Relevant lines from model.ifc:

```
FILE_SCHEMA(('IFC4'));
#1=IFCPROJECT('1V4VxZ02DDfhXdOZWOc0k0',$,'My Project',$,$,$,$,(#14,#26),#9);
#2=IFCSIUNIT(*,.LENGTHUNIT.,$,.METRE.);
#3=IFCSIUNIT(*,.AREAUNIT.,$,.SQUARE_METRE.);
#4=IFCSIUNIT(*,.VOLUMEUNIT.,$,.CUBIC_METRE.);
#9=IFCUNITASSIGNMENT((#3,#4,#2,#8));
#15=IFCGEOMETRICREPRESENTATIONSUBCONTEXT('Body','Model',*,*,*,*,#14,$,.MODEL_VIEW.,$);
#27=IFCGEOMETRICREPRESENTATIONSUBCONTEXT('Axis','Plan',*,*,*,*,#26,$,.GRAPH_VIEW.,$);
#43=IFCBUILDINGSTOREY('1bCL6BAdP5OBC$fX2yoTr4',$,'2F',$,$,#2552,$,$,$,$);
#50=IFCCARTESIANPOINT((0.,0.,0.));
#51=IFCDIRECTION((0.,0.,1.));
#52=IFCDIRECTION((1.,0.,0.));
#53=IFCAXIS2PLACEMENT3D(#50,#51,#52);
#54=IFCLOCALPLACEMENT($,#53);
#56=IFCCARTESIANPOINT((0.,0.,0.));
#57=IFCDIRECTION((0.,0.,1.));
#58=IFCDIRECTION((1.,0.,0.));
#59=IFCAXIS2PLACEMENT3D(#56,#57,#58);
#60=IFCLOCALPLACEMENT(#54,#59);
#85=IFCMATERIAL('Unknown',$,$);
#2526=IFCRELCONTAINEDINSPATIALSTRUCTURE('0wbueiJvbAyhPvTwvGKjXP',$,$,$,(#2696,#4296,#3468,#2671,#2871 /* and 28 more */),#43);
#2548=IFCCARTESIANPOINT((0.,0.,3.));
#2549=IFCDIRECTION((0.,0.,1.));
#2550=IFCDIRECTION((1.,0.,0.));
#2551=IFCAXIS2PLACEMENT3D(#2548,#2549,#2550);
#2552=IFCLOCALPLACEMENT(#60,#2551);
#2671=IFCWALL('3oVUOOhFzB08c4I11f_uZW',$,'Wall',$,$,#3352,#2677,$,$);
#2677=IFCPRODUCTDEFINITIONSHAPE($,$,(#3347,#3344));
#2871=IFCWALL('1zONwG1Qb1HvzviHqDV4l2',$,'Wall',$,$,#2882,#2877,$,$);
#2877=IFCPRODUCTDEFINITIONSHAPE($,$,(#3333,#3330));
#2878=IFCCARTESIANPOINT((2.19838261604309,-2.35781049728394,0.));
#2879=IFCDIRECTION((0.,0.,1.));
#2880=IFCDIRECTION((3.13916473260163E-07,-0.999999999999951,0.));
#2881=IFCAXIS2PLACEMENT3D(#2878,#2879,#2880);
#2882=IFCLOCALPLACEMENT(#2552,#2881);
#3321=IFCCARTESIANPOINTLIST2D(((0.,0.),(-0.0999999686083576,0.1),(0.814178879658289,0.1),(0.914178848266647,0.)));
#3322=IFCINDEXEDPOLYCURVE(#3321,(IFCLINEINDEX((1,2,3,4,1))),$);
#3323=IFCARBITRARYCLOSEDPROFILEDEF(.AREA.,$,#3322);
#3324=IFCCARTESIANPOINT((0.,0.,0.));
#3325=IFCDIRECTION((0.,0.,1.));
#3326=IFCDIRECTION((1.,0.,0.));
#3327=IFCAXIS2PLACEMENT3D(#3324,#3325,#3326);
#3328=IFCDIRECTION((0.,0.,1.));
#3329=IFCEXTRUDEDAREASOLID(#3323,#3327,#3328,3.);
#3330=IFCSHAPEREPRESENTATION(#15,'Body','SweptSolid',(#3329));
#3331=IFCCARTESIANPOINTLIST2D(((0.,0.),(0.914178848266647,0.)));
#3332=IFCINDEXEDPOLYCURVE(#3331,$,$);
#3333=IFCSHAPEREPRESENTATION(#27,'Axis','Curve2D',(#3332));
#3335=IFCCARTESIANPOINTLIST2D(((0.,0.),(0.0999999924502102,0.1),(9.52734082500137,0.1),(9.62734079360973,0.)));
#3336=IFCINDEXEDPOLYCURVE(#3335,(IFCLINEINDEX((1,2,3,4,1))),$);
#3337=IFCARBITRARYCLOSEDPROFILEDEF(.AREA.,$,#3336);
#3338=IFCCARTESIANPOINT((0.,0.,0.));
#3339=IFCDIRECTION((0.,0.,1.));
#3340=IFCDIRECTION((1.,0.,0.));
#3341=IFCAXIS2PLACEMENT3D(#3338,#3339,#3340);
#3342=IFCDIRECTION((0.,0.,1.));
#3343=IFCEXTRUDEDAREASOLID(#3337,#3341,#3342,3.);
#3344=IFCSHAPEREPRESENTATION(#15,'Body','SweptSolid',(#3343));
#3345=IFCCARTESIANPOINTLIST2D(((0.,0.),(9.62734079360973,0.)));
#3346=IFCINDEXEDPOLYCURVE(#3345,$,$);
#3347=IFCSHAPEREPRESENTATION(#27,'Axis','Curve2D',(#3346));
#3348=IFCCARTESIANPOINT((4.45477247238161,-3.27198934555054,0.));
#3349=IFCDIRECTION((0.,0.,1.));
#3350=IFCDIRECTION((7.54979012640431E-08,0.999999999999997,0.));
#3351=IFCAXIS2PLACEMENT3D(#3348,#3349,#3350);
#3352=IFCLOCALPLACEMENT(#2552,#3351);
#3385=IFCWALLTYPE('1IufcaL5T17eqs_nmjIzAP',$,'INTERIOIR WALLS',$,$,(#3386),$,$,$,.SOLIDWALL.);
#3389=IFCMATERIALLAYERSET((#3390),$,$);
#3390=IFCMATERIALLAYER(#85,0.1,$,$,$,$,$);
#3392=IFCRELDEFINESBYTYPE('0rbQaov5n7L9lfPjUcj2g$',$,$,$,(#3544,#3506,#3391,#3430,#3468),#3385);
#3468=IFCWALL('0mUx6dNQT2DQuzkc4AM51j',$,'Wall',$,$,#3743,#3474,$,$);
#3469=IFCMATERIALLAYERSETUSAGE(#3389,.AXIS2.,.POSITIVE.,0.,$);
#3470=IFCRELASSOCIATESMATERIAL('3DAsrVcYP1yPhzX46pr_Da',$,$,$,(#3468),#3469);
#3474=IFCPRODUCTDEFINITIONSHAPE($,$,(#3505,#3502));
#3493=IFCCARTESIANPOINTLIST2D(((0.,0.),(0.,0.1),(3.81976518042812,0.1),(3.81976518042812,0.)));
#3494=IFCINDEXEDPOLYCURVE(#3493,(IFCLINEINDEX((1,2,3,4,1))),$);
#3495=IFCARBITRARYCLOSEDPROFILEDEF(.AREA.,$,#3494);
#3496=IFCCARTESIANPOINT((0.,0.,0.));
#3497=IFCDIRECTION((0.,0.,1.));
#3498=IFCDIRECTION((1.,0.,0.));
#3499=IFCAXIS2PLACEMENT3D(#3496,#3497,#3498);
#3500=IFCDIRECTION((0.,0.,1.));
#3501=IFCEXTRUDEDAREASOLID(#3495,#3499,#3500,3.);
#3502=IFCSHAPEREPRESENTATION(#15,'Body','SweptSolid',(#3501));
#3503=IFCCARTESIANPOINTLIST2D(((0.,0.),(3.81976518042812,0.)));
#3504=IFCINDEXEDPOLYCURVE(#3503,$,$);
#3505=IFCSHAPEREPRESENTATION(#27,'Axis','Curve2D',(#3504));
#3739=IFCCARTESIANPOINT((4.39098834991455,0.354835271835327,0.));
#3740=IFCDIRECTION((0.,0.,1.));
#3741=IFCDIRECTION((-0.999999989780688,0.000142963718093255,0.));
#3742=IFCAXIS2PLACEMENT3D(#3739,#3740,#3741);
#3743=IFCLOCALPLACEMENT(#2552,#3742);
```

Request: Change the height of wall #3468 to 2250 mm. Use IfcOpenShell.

```python
import ifcopenshell
import ifcopenshell.geom
import ifcopenshell.util.representation
import ifcopenshell.util.shape
import ifcopenshell.util.unit

model = ifcopenshell.open("model.ifc")
unit_scale = ifcopenshell.util.unit.calculate_unit_scale(model)
settings = ifcopenshell.geom.settings()


def volume(element):
    """Net volume in cubic metres, openings subtracted."""
    shape = ifcopenshell.geom.create_shape(settings, element)
    return ifcopenshell.util.shape.get_volume(shape.geometry)


wall = model.by_guid("0mUx6dNQT2DQuzkc4AM51j")
before = volume(wall)

body = ifcopenshell.util.representation.get_representation(wall, "Model", "Body")
solid = body.Items[0]
old_height = solid.Depth
solid.Depth = 2.25 / unit_scale
after = volume(wall)

print(f"height {old_height:g} -> {solid.Depth:g}, volume {before:.3f} -> {after:.3f} m3")

model.write("model-out.ifc")
```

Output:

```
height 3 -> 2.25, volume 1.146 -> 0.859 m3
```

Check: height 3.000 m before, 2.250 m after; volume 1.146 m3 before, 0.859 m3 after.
